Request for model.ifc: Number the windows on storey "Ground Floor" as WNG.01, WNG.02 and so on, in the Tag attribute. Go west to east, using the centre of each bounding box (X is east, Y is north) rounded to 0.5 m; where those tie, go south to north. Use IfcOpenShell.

First a look at what the model holds.

```python
import ifcopenshell
import ifcopenshell.util.element
import ifcopenshell.util.placement

model = ifcopenshell.open("model.ifc")
print(model.schema)
storey = next(s for s in model.by_type("IfcBuildingStorey") if s.Name == "Ground Floor")
windows = [e for e in ifcopenshell.util.element.get_decomposition(storey) if e.is_a("IfcWindow")]
for e in sorted(windows, key=lambda e: e.id()):
    origin = ifcopenshell.util.placement.get_local_placement(e.ObjectPlacement)[:3, 3]
    print(e.id(), e.Tag, e.Name, origin.round(2) + 0.0, sep=" | ")
```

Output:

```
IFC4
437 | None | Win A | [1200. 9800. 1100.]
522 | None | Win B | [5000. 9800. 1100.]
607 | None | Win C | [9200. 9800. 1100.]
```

```python
import ifcopenshell
import ifcopenshell.geom
import ifcopenshell.util.element
import ifcopenshell.util.shape

model = ifcopenshell.open("model.ifc")
settings = ifcopenshell.geom.settings()
settings.set("use-world-coords", True)


def centre(element):
    shape = ifcopenshell.geom.create_shape(settings, element)
    return ifcopenshell.util.shape.get_bbox_centroid(shape.geometry)


storey = next(s for s in model.by_type("IfcBuildingStorey") if s.Name == "Ground Floor")
windows = [e for e in ifcopenshell.util.element.get_decomposition(storey) if e.is_a("IfcWindow")]

# Insertion points can sit at a corner or the storey origin, so sort by the geometry (in metres).
centres = {e: centre(e) for e in windows}
windows.sort(key=lambda e: (round(centres[e][0] / 0.5), centres[e][1]))

for i, e in enumerate(windows, start=1):
    number = f"WNG.{i:02d}"
    e.Tag = number
    print(e.id(), number)

model.write("model_rev.ifc")
```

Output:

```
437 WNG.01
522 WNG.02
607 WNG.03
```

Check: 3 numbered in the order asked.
